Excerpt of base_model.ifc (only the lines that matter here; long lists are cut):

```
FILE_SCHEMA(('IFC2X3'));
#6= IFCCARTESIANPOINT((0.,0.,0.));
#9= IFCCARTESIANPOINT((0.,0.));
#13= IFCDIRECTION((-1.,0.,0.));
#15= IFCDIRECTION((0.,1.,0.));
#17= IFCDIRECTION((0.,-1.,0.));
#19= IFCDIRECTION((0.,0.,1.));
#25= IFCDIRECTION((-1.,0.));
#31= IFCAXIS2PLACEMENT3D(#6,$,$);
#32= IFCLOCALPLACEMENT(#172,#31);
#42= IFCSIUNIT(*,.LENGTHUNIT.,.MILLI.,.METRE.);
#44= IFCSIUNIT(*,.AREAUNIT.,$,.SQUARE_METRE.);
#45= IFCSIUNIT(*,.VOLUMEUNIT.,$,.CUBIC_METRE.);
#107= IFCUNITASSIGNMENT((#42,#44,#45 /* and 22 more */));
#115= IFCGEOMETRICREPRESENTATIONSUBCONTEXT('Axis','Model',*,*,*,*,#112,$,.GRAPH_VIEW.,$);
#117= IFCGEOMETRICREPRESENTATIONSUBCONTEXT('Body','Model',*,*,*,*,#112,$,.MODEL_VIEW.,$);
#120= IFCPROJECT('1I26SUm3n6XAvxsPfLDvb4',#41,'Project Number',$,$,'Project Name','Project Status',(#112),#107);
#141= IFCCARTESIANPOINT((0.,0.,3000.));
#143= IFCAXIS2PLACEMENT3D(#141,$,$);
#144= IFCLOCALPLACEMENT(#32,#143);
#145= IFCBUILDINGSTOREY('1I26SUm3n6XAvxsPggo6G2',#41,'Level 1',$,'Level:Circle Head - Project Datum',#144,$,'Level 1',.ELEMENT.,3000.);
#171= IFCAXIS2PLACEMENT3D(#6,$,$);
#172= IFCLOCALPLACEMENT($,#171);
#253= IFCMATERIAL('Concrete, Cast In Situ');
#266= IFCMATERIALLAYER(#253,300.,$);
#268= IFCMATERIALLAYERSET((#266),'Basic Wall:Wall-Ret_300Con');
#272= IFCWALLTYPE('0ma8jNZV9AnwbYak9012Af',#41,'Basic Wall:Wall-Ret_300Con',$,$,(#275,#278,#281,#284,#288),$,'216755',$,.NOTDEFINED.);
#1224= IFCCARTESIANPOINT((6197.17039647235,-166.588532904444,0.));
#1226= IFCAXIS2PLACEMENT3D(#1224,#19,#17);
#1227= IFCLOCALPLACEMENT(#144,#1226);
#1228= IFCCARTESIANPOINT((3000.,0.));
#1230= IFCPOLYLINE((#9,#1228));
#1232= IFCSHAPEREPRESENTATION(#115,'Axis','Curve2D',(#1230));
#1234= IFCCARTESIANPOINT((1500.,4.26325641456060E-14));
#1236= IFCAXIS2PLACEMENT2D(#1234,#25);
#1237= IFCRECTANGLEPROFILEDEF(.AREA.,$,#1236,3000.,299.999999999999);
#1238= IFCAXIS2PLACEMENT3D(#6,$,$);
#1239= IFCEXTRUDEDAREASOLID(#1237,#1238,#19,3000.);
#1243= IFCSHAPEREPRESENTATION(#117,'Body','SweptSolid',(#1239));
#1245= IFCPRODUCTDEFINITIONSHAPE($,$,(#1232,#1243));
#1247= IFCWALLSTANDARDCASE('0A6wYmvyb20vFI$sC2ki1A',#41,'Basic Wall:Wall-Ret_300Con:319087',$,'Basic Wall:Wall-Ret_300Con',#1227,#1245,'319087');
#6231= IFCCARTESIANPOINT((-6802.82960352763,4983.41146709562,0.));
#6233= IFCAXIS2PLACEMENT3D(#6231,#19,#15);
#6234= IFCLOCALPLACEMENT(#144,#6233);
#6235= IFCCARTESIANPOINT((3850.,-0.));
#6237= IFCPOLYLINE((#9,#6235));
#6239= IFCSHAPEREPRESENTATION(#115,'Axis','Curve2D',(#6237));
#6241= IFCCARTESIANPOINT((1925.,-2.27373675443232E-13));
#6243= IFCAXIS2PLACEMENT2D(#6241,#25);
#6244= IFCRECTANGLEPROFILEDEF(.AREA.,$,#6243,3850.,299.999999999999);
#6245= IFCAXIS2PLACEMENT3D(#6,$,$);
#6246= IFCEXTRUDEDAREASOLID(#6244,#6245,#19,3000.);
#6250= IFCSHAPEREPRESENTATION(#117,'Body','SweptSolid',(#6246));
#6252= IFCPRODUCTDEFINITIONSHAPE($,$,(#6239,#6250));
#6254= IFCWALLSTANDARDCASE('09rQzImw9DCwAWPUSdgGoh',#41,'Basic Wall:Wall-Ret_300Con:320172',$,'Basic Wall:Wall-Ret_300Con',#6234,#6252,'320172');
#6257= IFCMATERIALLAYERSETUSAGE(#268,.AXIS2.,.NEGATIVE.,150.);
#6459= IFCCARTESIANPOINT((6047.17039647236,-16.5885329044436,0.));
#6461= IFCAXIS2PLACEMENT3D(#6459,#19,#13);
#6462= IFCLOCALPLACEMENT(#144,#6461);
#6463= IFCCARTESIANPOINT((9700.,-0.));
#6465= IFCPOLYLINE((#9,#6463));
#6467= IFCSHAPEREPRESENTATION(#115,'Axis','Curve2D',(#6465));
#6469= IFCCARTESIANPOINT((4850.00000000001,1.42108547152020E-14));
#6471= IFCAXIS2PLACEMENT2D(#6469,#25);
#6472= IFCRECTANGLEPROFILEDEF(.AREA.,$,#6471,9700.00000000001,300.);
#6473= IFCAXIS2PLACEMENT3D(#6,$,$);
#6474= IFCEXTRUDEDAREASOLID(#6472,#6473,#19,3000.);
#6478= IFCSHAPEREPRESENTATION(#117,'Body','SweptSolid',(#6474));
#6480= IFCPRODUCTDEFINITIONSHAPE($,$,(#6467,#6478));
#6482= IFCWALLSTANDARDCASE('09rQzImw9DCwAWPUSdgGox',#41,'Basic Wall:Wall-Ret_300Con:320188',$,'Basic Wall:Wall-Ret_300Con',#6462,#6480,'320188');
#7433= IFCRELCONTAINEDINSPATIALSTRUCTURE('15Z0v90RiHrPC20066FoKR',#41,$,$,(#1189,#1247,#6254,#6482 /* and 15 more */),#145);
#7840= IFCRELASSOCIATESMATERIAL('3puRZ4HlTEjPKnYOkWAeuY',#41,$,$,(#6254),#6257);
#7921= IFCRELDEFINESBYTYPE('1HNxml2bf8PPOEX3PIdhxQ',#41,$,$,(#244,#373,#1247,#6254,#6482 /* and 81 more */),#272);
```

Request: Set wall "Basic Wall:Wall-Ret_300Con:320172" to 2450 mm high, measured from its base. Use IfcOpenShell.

```python
import ifcopenshell
import ifcopenshell.geom
import ifcopenshell.util.representation
import ifcopenshell.util.shape

model = ifcopenshell.open("base_model.ifc")
settings = ifcopenshell.geom.settings()


def volume(element):
    """Net volume in cubic metres, openings subtracted."""
    shape = ifcopenshell.geom.create_shape(settings, element)
    return ifcopenshell.util.shape.get_volume(shape.geometry)


wall = model.by_guid("09rQzImw9DCwAWPUSdgGoh")
before = volume(wall)

body = ifcopenshell.util.representation.get_representation(wall, "Model", "Body")
solid = body.Items[0]
old_height = solid.Depth
solid.Depth = 2450.0
after = volume(wall)

print(f"height {old_height:g} -> {solid.Depth:g}, volume {before:.3f} -> {after:.3f} m3")

model.write("base_model-out.ifc")
```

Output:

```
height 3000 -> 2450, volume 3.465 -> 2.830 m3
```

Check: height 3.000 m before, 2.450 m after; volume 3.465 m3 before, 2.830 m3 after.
